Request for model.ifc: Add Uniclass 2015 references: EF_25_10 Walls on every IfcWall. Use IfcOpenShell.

First a look at what the model holds.

```python
import ifcopenshell

model = ifcopenshell.open("model.ifc")
print(model.schema)
print("classifications:", [c.Name for c in model.by_type("IfcClassification")])
for ifc_class in ("IfcDoor", "IfcRoof", "IfcStair", "IfcWall", "IfcWindow"):
    print(ifc_class, len(model.by_type(ifc_class)))
```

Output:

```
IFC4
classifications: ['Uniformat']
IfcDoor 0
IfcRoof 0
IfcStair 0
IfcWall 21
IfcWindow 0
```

```python
import ifcopenshell
import ifcopenshell.api.classification

model = ifcopenshell.open("model.ifc")

system = ifcopenshell.api.classification.add_classification(model, classification="Uniclass 2015")

codes = {
    "IfcWall": ("EF_25_10", "Walls"),
}
for ifc_class, (code, name) in codes.items():
    products = model.by_type(ifc_class)
    ifcopenshell.api.classification.add_reference(
        model, products=products, classification=system, identification=code, name=name
    )
    print(code, len(products))

model.write("model-out.ifc")
```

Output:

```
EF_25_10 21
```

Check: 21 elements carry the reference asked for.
